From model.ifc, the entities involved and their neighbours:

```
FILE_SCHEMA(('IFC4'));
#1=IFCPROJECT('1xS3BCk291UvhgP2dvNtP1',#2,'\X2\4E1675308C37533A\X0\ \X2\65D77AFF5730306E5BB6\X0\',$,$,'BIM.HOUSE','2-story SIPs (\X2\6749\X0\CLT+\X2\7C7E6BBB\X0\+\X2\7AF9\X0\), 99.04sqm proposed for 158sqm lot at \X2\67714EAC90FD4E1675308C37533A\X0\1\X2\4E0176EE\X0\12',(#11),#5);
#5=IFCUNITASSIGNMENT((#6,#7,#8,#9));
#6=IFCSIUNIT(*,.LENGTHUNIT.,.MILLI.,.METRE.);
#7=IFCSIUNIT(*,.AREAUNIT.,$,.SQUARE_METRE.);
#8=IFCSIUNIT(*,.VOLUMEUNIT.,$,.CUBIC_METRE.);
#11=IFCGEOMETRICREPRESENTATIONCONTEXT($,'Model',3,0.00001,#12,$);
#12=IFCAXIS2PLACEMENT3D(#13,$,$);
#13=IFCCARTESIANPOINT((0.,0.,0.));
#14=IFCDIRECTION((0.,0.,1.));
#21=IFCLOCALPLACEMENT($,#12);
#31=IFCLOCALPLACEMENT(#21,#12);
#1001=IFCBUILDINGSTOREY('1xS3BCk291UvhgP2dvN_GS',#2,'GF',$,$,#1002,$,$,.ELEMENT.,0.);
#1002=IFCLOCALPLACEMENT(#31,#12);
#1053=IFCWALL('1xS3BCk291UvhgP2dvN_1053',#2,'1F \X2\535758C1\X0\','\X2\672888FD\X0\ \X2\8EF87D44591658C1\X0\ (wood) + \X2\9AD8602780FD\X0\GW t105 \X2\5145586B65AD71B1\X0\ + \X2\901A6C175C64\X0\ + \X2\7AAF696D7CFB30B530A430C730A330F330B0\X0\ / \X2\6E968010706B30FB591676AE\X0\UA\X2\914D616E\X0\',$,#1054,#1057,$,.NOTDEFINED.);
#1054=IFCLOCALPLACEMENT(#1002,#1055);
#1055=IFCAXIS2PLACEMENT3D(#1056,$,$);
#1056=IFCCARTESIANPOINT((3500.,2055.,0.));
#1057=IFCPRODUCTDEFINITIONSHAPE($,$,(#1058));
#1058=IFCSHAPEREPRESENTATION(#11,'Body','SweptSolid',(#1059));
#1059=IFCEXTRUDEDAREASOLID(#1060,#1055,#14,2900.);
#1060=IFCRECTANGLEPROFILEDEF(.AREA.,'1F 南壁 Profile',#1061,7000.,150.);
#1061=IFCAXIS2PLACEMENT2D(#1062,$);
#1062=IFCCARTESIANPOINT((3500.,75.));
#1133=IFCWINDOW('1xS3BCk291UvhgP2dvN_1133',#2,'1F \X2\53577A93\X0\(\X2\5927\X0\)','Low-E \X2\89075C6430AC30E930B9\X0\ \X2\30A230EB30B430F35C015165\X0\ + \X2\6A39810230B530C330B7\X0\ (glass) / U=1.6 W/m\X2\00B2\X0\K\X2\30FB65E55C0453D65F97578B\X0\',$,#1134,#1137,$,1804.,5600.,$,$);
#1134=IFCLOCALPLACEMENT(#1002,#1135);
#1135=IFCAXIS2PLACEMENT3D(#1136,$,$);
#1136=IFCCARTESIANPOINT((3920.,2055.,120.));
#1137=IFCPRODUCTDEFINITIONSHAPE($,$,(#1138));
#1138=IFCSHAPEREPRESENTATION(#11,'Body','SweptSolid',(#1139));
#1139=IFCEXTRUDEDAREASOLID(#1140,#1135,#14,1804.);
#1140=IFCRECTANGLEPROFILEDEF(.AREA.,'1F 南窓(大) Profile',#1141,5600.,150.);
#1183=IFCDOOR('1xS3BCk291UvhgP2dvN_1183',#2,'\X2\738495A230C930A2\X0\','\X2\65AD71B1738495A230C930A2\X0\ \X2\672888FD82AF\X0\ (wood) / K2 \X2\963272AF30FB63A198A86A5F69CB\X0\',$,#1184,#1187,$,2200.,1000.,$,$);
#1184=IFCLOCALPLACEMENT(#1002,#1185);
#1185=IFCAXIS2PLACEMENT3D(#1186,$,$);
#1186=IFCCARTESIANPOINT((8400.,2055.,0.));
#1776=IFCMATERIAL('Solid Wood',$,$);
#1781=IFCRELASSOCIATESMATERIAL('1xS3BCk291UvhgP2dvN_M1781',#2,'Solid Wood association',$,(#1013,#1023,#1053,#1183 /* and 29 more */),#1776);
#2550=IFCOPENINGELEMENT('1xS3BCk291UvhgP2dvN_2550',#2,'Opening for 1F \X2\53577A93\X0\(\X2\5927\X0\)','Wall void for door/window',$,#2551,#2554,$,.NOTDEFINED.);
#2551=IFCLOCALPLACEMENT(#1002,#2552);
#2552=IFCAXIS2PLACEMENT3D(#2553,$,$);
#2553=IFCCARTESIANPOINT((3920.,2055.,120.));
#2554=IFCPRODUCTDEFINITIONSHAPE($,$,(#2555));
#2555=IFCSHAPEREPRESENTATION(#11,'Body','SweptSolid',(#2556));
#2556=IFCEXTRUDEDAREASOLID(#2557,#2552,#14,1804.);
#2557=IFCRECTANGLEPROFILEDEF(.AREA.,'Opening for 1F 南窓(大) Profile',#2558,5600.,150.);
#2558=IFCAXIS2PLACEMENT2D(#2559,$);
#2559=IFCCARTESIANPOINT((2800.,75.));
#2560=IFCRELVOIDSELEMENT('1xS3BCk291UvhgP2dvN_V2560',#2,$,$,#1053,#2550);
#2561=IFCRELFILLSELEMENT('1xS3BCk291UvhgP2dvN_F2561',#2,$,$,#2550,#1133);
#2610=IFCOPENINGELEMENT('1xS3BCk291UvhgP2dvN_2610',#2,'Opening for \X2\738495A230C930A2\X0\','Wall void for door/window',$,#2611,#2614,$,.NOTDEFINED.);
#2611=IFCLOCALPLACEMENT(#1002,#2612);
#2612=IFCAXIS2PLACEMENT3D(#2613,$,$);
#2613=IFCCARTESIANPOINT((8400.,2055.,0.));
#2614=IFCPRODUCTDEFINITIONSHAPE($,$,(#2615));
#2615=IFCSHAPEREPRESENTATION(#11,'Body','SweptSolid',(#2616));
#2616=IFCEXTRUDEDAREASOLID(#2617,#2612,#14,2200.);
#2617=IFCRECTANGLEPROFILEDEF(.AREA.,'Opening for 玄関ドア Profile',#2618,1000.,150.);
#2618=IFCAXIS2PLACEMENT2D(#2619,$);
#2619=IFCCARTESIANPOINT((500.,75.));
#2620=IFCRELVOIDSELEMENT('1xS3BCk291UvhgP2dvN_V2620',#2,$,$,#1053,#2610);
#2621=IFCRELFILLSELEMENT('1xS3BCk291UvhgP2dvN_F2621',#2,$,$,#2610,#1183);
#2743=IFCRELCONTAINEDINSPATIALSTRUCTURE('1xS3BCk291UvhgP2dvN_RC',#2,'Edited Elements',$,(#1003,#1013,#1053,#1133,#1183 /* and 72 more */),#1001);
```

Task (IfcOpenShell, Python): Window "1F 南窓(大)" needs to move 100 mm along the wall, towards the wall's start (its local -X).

```python
import ifcopenshell
import ifcopenshell.api.geometry
import ifcopenshell.util.placement
import ifcopenshell.util.unit

model = ifcopenshell.open("model.ifc")
unit_scale = ifcopenshell.util.unit.calculate_unit_scale(model)

window = model.by_id(1133)
opening = window.FillsVoids[0].RelatingOpeningElement
wall = opening.VoidsElements[0].RelatingBuildingElement

wall_matrix = ifcopenshell.util.placement.get_local_placement(wall.ObjectPlacement)
shift = wall_matrix[:3, 0] * -0.1 / unit_scale
before = ifcopenshell.util.placement.get_local_placement(window.ObjectPlacement)[:3, 3].copy()

# The window is not placed relative to its opening, so move both.
for product in (opening, window):
    matrix = ifcopenshell.util.placement.get_local_placement(product.ObjectPlacement)
    matrix[:3, 3] += shift
    ifcopenshell.api.geometry.edit_object_placement(model, product=product, matrix=matrix, is_si=False)

after = ifcopenshell.util.placement.get_local_placement(window.ObjectPlacement)[:3, 3]
print("window moved by", (after - before).round(3) + 0.0)

model.write("model_updated.ifc")
```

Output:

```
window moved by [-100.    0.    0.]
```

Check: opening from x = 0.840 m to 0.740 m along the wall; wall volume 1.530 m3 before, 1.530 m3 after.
